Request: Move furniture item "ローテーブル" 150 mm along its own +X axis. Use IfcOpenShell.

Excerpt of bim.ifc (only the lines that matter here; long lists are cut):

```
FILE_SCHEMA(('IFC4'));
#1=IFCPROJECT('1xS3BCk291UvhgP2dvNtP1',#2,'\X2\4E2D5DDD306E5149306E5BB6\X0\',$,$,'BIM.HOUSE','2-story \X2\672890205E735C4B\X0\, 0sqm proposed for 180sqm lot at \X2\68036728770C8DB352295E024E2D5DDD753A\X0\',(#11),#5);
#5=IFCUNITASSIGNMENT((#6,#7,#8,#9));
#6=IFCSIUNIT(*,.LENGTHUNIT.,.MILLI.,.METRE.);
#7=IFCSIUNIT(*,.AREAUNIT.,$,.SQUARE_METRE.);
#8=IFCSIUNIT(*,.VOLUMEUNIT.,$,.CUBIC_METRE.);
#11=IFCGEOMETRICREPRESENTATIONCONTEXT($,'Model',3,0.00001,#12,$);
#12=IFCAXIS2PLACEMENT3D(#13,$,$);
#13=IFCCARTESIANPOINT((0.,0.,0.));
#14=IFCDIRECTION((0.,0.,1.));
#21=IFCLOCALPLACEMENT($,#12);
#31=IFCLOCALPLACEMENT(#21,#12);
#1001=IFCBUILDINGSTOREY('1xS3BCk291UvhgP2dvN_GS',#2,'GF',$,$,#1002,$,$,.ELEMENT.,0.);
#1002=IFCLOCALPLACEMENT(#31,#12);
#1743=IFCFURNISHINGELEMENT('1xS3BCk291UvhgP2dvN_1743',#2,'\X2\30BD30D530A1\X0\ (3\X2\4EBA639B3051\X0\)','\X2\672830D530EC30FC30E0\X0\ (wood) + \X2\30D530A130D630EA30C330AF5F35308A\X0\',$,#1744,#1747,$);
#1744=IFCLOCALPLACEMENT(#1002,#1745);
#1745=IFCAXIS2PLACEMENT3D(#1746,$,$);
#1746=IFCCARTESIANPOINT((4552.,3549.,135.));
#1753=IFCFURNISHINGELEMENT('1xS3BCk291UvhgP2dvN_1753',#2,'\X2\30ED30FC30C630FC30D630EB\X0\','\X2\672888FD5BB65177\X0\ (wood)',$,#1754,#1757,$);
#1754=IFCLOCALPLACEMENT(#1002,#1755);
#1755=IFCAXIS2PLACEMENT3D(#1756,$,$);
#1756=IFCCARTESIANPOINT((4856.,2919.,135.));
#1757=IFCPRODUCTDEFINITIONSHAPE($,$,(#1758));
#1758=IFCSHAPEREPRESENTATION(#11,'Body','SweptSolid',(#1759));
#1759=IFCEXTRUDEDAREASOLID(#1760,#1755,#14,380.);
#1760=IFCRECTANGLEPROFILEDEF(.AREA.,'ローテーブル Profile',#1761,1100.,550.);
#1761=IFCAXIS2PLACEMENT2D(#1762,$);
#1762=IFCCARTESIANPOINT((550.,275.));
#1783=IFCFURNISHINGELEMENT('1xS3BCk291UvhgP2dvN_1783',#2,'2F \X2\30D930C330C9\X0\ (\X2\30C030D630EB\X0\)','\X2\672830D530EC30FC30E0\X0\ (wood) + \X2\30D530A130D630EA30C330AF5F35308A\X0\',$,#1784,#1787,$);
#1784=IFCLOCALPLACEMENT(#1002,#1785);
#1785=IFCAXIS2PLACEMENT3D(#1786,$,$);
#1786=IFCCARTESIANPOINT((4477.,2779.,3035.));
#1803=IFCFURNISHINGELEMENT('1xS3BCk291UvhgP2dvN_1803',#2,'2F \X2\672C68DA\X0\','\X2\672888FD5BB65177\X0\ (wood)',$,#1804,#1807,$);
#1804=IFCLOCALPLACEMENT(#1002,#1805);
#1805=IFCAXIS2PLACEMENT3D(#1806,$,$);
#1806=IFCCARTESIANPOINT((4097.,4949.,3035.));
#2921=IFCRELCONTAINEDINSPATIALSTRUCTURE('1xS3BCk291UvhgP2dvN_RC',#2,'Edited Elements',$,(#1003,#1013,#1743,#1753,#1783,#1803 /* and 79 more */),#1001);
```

```python
import ifcopenshell
import ifcopenshell.api.geometry
import ifcopenshell.util.placement
import ifcopenshell.util.unit

model = ifcopenshell.open("bim.ifc")
unit_scale = ifcopenshell.util.unit.calculate_unit_scale(model)

item = model.by_guid("1xS3BCk291UvhgP2dvN_1753")
matrix = ifcopenshell.util.placement.get_local_placement(item.ObjectPlacement)
matrix[:3, 3] += matrix[:3, 0] * 0.15 / unit_scale
ifcopenshell.api.geometry.edit_object_placement(model, product=item, matrix=matrix, is_si=False)

print(ifcopenshell.util.placement.get_local_placement(item.ObjectPlacement).round(3) + 0.0)

model.write("bim-out.ifc")
```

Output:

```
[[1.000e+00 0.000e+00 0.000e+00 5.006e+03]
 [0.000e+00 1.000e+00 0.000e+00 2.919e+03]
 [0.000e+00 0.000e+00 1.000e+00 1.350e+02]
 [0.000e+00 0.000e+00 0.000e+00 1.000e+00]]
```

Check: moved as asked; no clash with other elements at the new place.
